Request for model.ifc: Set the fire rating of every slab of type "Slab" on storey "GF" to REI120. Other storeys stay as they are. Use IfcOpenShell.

First a look at what the model holds.

```python
import ifcopenshell
import ifcopenshell.util.element

model = ifcopenshell.open("model.ifc")
print(model.schema)
storey = next(s for s in model.by_type("IfcBuildingStorey") if s.Name == "GF")
slabs = [e for e in ifcopenshell.util.element.get_decomposition(storey) if e.is_a("IfcSlab")]
seen = {}
for e in slabs:
    element_type = ifcopenshell.util.element.get_type(e)
    key = (element_type.Name if element_type != e and element_type else None, ifcopenshell.util.element.get_pset(e, "Pset_SlabCommon", "FireRating"))
    seen[key] = seen.get(key, 0) + 1
for (name, value), count in sorted(seen.items(), key=str):
    print(count, "x", name, "|", value)
```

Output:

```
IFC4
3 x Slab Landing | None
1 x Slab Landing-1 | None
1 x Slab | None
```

```python
import ifcopenshell
import ifcopenshell.api.pset
import ifcopenshell.util.element

model = ifcopenshell.open("model.ifc")

storey = next(s for s in model.by_type("IfcBuildingStorey") if s.Name == "GF")
slabs = [e for e in ifcopenshell.util.element.get_decomposition(storey) if e.is_a("IfcSlab")]

count = 0
for e in slabs:
    element_type = ifcopenshell.util.element.get_type(e)
    if element_type in (None, e) or element_type.Name != "Slab":
        continue
    # add_pset returns the element's existing set when there is one.
    pset = ifcopenshell.api.pset.add_pset(model, product=e, name="Pset_SlabCommon")
    ifcopenshell.api.pset.edit_pset(model, pset=pset, properties={"FireRating": "REI120"})
    count += 1

print(count, "slabs updated")

model.write("model_v2.ifc")
```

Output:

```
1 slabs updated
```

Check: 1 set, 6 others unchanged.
